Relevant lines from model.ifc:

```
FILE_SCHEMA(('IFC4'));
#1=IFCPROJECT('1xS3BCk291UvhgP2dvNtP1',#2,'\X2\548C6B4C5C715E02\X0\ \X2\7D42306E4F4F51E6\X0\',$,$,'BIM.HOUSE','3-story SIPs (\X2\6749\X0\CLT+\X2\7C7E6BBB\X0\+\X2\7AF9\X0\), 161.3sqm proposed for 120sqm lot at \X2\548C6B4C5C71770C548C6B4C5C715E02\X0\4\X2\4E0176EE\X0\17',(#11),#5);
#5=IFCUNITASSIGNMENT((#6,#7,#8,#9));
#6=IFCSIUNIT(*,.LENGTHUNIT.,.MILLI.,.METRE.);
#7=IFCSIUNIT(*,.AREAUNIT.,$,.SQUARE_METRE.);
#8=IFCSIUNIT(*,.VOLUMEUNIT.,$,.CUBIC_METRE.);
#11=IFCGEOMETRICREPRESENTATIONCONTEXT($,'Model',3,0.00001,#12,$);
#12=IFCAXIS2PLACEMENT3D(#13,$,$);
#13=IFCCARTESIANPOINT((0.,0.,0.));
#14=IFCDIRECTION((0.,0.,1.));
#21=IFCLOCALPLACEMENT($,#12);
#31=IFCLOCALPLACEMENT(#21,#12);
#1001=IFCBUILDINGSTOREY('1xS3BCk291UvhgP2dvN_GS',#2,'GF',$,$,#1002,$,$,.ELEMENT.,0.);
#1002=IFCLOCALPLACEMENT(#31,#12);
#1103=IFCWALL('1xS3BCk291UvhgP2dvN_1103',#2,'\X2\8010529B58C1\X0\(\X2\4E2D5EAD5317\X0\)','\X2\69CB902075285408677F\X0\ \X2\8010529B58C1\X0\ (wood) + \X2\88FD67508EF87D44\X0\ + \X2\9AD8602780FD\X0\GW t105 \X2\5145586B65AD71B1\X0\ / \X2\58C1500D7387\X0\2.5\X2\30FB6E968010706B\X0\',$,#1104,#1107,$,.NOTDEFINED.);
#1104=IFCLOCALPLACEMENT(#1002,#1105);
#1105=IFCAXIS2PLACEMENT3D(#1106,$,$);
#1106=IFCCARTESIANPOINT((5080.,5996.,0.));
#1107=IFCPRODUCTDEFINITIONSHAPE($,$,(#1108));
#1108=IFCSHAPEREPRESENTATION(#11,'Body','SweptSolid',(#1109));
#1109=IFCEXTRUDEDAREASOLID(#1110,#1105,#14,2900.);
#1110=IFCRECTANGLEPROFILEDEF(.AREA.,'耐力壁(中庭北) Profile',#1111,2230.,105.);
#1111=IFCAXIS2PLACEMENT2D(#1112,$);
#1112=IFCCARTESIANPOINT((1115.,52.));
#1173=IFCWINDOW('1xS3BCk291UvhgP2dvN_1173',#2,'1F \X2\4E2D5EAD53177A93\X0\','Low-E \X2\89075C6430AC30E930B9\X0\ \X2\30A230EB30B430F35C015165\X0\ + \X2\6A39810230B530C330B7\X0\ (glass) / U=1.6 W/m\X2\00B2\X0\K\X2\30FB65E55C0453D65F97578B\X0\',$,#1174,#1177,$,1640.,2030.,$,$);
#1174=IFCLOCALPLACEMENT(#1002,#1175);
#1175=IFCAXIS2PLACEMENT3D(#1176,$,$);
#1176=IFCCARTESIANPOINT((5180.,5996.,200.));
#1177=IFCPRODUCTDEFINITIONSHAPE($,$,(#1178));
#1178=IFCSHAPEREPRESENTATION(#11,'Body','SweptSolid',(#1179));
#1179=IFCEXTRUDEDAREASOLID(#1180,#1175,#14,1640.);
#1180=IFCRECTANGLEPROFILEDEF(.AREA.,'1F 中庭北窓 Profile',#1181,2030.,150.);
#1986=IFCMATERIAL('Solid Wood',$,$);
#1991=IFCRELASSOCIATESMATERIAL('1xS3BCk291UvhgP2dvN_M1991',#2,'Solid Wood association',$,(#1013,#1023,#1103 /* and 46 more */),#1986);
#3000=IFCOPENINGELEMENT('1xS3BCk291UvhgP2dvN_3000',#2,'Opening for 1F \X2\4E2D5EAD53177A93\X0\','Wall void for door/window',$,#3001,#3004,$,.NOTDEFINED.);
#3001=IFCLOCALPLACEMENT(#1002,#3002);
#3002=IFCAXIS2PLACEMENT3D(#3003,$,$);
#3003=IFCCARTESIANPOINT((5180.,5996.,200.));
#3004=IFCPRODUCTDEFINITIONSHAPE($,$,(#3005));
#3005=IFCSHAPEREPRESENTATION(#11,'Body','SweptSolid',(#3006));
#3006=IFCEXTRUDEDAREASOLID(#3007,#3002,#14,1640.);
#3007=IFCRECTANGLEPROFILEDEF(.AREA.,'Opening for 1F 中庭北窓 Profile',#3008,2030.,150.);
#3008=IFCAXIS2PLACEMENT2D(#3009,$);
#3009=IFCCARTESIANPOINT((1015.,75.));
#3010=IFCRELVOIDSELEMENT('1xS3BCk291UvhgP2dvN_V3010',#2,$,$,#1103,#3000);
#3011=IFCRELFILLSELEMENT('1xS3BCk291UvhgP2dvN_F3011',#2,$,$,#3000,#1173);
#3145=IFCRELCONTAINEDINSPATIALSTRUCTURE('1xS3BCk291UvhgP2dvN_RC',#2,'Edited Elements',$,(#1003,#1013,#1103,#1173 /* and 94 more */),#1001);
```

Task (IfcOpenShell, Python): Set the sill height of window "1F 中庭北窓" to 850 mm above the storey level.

```python
import numpy as np
import ifcopenshell
import ifcopenshell.api.geometry
import ifcopenshell.geom
import ifcopenshell.util.element
import ifcopenshell.util.placement
import ifcopenshell.util.shape
import ifcopenshell.util.unit

model = ifcopenshell.open("model.ifc")
unit_scale = ifcopenshell.util.unit.calculate_unit_scale(model)

window = model.by_guid("1xS3BCk291UvhgP2dvN_1173")
opening = window.FillsVoids[0].RelatingOpeningElement
storey = ifcopenshell.util.element.get_container(window, ifc_class="IfcBuildingStorey")
level = ifcopenshell.util.placement.get_local_placement(storey.ObjectPlacement)[2, 3]

# The opening's origin need not be at the sill, so measure its lowest point.
shape = ifcopenshell.geom.create_shape(ifcopenshell.geom.settings(), opening)
bottom = ifcopenshell.util.shape.get_shape_bottom_elevation(shape, shape.geometry) / unit_scale
dz = level + 0.85 / unit_scale - bottom

shift = np.array([0.0, 0.0, dz])
# The window is not placed relative to its opening, so move both.
for product in (opening, window):
    matrix = ifcopenshell.util.placement.get_local_placement(product.ObjectPlacement)
    matrix[:3, 3] += shift
    ifcopenshell.api.geometry.edit_object_placement(model, product=product, matrix=matrix, is_si=False)

print(f"moved by {dz * unit_scale:+.3f} m")

model.write("model_rev.ifc")
```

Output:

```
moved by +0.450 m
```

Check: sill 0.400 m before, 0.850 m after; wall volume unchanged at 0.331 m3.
